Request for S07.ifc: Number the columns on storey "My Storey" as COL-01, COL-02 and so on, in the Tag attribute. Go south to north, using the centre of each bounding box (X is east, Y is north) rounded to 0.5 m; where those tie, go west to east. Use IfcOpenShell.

First a look at what the model holds.

```python
import ifcopenshell
import ifcopenshell.util.element
import ifcopenshell.util.placement

model = ifcopenshell.open("S07.ifc")
print(model.schema)
storey = next(s for s in model.by_type("IfcBuildingStorey") if s.Name == "My Storey")
columns = [e for e in ifcopenshell.util.element.get_decomposition(storey) if e.is_a("IfcColumn")]
for e in sorted(columns, key=lambda e: e.id()):
    origin = ifcopenshell.util.placement.get_local_placement(e.ObjectPlacement)[:3, 3]
    print(e.id(), e.Tag, e.Name, origin.round(2) + 0.0, sep=" | ")
```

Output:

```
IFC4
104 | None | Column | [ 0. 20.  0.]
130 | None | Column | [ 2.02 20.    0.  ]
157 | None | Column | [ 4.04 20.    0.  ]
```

```python
import ifcopenshell
import ifcopenshell.geom
import ifcopenshell.util.element
import ifcopenshell.util.shape

model = ifcopenshell.open("S07.ifc")
settings = ifcopenshell.geom.settings()
settings.set("use-world-coords", True)


def centre(element):
    shape = ifcopenshell.geom.create_shape(settings, element)
    return ifcopenshell.util.shape.get_bbox_centroid(shape.geometry)


storey = next(s for s in model.by_type("IfcBuildingStorey") if s.Name == "My Storey")
columns = [e for e in ifcopenshell.util.element.get_decomposition(storey) if e.is_a("IfcColumn")]

# Insertion points can sit at a corner or the storey origin, so sort by the geometry (in metres).
centres = {e: centre(e) for e in columns}
columns.sort(key=lambda e: (round(centres[e][1] / 0.5), centres[e][0]))

for i, e in enumerate(columns, start=1):
    number = f"COL-{i:02d}"
    e.Tag = number
    print(e.id(), number)

model.write("S07_edited.ifc")
```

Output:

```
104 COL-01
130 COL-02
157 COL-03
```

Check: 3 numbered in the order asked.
